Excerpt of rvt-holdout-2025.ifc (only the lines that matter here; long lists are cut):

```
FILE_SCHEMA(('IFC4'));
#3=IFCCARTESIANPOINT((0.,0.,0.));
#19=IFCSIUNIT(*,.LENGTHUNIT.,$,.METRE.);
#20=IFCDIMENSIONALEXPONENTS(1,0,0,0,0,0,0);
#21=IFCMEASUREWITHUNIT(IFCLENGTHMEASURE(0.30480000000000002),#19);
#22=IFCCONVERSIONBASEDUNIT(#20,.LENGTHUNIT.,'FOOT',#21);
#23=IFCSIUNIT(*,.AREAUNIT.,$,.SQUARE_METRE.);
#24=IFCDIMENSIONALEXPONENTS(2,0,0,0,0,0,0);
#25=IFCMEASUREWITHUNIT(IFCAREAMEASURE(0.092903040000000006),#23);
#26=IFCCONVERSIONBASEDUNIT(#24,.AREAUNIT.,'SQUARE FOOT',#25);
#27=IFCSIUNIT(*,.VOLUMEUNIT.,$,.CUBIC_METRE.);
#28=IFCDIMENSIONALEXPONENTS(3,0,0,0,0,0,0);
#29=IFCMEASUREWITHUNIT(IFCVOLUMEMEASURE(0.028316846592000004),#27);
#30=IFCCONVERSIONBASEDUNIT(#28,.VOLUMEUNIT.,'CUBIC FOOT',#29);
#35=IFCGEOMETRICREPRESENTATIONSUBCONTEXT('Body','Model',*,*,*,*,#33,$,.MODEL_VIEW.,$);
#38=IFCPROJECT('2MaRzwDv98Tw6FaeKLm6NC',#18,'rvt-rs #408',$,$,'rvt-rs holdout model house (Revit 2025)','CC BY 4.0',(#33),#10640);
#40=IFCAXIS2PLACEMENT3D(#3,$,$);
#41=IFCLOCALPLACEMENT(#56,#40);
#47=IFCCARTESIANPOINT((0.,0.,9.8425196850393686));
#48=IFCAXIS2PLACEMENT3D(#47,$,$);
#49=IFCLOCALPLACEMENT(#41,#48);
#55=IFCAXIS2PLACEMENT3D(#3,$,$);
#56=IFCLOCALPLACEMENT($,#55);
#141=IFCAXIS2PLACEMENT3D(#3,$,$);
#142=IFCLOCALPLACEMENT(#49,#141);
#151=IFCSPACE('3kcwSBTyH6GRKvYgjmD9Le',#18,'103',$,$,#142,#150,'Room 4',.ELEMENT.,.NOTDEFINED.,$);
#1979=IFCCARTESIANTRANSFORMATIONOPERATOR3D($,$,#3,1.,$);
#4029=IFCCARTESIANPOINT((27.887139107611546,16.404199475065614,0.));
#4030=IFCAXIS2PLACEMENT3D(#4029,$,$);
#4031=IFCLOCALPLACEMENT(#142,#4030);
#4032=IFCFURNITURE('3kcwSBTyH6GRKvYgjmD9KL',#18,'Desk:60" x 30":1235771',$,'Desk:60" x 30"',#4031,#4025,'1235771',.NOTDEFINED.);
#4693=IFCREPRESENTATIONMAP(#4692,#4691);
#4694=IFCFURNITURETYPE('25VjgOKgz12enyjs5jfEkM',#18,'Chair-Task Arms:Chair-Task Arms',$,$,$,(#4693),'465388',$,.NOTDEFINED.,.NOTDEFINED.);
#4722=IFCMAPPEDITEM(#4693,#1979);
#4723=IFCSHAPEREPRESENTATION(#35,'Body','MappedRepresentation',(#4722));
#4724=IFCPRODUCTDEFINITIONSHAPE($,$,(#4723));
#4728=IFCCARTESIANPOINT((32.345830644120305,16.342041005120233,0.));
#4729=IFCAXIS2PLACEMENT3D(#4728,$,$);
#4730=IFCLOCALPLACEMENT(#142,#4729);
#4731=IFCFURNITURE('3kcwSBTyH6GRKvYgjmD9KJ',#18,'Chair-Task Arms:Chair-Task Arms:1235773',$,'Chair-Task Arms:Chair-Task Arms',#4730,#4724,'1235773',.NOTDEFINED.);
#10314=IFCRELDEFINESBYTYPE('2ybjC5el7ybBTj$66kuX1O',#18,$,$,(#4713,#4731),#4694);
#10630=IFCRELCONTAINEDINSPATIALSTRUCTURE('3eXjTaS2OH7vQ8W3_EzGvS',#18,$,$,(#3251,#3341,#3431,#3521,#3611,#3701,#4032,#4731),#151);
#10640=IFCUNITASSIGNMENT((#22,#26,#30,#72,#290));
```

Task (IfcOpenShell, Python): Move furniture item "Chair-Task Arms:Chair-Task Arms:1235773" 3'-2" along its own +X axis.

```python
import ifcopenshell
import ifcopenshell.api.geometry
import ifcopenshell.util.placement
import ifcopenshell.util.unit

model = ifcopenshell.open("rvt-holdout-2025.ifc")
unit_scale = ifcopenshell.util.unit.calculate_unit_scale(model)

item = model.by_id(4731)
matrix = ifcopenshell.util.placement.get_local_placement(item.ObjectPlacement)
matrix[:3, 3] += matrix[:3, 0] * 38 * 0.0254 / unit_scale
ifcopenshell.api.geometry.edit_object_placement(model, product=item, matrix=matrix, is_si=False)

print(ifcopenshell.util.placement.get_local_placement(item.ObjectPlacement).round(3) + 0.0)

model.write("rvt-holdout-2025-out.ifc")
```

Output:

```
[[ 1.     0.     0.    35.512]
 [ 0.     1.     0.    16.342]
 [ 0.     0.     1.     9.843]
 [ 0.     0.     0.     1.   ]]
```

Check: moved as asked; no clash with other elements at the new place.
